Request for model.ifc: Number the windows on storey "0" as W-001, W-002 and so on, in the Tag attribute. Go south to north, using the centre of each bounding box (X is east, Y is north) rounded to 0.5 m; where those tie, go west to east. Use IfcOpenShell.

First a look at what the model holds.

```python
import ifcopenshell
import ifcopenshell.util.element
import ifcopenshell.util.placement

model = ifcopenshell.open("model.ifc")
print(model.schema)
storey = next(s for s in model.by_type("IfcBuildingStorey") if s.Name == "0")
windows = [e for e in ifcopenshell.util.element.get_decomposition(storey) if e.is_a("IfcWindow")]
for e in sorted(windows, key=lambda e: e.id()):
    origin = ifcopenshell.util.placement.get_local_placement(e.ObjectPlacement)[:3, 3]
    print(e.id(), e.Tag, e.Name, origin.round(2) + 0.0, sep=" | ")
```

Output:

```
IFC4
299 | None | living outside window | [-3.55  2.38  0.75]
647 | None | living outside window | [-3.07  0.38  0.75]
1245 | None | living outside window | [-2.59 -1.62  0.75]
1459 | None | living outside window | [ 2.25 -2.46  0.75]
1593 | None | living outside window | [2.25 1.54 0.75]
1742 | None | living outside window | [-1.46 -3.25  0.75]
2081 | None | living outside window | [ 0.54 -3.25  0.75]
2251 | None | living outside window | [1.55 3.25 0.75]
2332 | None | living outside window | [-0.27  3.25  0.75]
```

```python
import ifcopenshell
import ifcopenshell.geom
import ifcopenshell.util.element
import ifcopenshell.util.shape

model = ifcopenshell.open("model.ifc")
settings = ifcopenshell.geom.settings()
settings.set("use-world-coords", True)


def centre(element):
    shape = ifcopenshell.geom.create_shape(settings, element)
    return ifcopenshell.util.shape.get_bbox_centroid(shape.geometry)


storey = next(s for s in model.by_type("IfcBuildingStorey") if s.Name == "0")
windows = [e for e in ifcopenshell.util.element.get_decomposition(storey) if e.is_a("IfcWindow")]

# Insertion points can sit at a corner or the storey origin, so sort by the geometry (in metres).
centres = {e: centre(e) for e in windows}
windows.sort(key=lambda e: (round(centres[e][1] / 0.5), centres[e][0]))

for i, e in enumerate(windows, start=1):
    number = f"W-0{i:02d}"
    e.Tag = number
    print(e.id(), number)

model.write("model_rev.ifc")
```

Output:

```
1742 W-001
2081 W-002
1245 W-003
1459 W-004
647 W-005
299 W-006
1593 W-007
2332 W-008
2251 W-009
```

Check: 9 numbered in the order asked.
